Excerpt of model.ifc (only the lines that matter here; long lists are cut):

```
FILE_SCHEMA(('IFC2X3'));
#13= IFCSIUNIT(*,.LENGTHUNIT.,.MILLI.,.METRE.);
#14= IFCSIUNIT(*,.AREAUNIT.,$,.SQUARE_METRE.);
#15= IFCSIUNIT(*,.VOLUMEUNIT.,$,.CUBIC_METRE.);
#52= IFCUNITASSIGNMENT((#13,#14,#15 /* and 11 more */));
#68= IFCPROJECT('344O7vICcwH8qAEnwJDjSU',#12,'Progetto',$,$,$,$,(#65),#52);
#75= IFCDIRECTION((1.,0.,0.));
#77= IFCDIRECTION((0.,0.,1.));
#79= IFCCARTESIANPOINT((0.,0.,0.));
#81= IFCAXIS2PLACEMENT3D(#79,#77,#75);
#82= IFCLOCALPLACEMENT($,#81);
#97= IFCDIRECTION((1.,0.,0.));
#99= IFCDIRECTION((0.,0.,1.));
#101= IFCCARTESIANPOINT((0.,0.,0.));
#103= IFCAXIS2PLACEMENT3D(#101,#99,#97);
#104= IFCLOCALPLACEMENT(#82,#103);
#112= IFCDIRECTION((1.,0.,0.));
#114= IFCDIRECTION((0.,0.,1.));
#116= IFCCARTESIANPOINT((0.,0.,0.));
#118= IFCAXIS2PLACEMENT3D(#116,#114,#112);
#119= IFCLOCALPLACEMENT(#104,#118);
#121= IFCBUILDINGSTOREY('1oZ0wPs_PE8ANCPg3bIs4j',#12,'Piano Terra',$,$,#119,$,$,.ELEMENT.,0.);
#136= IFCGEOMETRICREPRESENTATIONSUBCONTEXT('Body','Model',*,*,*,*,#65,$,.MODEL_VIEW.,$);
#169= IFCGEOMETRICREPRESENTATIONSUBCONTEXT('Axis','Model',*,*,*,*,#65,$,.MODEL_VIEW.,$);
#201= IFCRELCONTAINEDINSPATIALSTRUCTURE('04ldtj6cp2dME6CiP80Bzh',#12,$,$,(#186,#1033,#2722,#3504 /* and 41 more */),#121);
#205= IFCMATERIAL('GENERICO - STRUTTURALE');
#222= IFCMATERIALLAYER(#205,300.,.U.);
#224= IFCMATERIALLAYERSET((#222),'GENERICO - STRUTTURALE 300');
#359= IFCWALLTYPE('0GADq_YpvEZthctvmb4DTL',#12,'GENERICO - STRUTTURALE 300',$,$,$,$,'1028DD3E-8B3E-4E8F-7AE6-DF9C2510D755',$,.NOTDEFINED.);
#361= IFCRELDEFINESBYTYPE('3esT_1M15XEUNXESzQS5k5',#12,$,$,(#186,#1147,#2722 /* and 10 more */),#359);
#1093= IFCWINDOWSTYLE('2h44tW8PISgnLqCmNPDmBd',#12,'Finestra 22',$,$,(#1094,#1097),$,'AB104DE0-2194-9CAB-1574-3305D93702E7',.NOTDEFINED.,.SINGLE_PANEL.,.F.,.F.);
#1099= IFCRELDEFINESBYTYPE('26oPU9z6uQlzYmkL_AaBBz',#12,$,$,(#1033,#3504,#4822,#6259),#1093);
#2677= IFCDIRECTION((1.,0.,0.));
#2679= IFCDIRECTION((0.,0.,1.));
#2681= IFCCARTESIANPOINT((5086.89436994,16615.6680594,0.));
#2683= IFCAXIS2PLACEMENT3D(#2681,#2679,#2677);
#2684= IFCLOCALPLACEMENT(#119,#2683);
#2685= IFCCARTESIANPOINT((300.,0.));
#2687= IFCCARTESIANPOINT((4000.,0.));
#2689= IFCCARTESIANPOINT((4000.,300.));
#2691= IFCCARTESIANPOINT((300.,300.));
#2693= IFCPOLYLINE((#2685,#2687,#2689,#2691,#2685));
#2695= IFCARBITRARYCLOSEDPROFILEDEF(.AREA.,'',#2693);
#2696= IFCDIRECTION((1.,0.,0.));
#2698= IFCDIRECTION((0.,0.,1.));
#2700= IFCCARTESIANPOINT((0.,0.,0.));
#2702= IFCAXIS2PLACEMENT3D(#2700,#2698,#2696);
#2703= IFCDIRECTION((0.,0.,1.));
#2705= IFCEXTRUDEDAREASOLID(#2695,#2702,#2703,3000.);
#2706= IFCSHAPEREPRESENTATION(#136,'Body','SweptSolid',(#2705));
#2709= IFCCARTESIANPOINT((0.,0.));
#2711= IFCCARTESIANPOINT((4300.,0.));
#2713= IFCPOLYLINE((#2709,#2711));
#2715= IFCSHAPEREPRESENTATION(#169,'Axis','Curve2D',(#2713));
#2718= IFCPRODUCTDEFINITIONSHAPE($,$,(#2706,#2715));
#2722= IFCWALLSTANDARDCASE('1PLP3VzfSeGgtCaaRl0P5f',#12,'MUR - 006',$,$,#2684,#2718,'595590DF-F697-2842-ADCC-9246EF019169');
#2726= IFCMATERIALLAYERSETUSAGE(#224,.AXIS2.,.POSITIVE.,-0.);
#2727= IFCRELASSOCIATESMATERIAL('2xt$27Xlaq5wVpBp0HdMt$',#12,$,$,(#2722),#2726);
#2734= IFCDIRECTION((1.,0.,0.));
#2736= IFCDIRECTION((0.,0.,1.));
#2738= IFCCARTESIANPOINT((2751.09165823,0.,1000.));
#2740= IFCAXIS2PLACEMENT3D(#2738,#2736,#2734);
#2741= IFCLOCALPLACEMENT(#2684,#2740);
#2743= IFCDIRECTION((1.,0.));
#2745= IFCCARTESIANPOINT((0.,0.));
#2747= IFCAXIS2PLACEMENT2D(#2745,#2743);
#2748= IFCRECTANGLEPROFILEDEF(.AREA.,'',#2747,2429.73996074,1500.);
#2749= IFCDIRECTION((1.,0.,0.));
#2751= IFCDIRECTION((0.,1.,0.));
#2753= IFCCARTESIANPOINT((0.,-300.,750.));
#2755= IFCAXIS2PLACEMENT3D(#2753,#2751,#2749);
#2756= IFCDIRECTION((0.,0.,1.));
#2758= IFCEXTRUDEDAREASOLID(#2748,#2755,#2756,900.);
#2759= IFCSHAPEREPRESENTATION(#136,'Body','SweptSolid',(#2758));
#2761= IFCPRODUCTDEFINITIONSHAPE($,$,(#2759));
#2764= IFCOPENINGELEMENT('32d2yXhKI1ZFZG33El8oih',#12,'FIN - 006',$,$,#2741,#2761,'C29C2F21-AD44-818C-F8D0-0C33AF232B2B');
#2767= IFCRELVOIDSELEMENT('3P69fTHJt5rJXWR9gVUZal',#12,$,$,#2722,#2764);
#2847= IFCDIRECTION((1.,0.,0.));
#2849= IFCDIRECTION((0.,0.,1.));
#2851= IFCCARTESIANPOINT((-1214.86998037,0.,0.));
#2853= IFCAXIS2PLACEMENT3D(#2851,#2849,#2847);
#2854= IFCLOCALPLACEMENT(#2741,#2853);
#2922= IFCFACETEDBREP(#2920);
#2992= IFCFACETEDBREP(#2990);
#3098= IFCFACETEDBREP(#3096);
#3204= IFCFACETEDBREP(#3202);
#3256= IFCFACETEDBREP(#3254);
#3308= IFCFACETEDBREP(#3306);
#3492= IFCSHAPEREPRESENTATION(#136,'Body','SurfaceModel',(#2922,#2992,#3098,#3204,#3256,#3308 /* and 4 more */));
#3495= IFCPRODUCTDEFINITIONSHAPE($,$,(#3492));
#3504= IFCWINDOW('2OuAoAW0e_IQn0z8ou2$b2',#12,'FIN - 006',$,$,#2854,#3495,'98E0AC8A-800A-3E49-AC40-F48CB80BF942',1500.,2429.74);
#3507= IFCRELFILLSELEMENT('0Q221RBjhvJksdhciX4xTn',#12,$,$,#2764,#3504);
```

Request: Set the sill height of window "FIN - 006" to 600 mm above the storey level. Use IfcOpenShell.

```python
import numpy as np
import ifcopenshell
import ifcopenshell.api.geometry
import ifcopenshell.geom
import ifcopenshell.util.element
import ifcopenshell.util.placement
import ifcopenshell.util.shape
import ifcopenshell.util.unit

model = ifcopenshell.open("model.ifc")
unit_scale = ifcopenshell.util.unit.calculate_unit_scale(model)

window = model.by_guid("2OuAoAW0e_IQn0z8ou2$b2")
opening = window.FillsVoids[0].RelatingOpeningElement
storey = ifcopenshell.util.element.get_container(window, ifc_class="IfcBuildingStorey")
level = ifcopenshell.util.placement.get_local_placement(storey.ObjectPlacement)[2, 3]

# The opening's origin need not be at the sill, so measure its lowest point.
shape = ifcopenshell.geom.create_shape(ifcopenshell.geom.settings(), opening)
bottom = ifcopenshell.util.shape.get_shape_bottom_elevation(shape, shape.geometry) / unit_scale
dz = level + 600.0 - bottom

shift = np.array([0.0, 0.0, dz])
# The window is placed relative to its opening, so it follows when the opening moves.
matrix = ifcopenshell.util.placement.get_local_placement(opening.ObjectPlacement)
matrix[:3, 3] += shift
ifcopenshell.api.geometry.edit_object_placement(
    model, product=opening, matrix=matrix, is_si=False, should_transform_children=True
)

print(f"moved by {dz * unit_scale:+.3f} m")

model.write("model_rev.ifc")
```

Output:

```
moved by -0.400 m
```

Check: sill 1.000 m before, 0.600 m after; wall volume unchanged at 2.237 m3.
